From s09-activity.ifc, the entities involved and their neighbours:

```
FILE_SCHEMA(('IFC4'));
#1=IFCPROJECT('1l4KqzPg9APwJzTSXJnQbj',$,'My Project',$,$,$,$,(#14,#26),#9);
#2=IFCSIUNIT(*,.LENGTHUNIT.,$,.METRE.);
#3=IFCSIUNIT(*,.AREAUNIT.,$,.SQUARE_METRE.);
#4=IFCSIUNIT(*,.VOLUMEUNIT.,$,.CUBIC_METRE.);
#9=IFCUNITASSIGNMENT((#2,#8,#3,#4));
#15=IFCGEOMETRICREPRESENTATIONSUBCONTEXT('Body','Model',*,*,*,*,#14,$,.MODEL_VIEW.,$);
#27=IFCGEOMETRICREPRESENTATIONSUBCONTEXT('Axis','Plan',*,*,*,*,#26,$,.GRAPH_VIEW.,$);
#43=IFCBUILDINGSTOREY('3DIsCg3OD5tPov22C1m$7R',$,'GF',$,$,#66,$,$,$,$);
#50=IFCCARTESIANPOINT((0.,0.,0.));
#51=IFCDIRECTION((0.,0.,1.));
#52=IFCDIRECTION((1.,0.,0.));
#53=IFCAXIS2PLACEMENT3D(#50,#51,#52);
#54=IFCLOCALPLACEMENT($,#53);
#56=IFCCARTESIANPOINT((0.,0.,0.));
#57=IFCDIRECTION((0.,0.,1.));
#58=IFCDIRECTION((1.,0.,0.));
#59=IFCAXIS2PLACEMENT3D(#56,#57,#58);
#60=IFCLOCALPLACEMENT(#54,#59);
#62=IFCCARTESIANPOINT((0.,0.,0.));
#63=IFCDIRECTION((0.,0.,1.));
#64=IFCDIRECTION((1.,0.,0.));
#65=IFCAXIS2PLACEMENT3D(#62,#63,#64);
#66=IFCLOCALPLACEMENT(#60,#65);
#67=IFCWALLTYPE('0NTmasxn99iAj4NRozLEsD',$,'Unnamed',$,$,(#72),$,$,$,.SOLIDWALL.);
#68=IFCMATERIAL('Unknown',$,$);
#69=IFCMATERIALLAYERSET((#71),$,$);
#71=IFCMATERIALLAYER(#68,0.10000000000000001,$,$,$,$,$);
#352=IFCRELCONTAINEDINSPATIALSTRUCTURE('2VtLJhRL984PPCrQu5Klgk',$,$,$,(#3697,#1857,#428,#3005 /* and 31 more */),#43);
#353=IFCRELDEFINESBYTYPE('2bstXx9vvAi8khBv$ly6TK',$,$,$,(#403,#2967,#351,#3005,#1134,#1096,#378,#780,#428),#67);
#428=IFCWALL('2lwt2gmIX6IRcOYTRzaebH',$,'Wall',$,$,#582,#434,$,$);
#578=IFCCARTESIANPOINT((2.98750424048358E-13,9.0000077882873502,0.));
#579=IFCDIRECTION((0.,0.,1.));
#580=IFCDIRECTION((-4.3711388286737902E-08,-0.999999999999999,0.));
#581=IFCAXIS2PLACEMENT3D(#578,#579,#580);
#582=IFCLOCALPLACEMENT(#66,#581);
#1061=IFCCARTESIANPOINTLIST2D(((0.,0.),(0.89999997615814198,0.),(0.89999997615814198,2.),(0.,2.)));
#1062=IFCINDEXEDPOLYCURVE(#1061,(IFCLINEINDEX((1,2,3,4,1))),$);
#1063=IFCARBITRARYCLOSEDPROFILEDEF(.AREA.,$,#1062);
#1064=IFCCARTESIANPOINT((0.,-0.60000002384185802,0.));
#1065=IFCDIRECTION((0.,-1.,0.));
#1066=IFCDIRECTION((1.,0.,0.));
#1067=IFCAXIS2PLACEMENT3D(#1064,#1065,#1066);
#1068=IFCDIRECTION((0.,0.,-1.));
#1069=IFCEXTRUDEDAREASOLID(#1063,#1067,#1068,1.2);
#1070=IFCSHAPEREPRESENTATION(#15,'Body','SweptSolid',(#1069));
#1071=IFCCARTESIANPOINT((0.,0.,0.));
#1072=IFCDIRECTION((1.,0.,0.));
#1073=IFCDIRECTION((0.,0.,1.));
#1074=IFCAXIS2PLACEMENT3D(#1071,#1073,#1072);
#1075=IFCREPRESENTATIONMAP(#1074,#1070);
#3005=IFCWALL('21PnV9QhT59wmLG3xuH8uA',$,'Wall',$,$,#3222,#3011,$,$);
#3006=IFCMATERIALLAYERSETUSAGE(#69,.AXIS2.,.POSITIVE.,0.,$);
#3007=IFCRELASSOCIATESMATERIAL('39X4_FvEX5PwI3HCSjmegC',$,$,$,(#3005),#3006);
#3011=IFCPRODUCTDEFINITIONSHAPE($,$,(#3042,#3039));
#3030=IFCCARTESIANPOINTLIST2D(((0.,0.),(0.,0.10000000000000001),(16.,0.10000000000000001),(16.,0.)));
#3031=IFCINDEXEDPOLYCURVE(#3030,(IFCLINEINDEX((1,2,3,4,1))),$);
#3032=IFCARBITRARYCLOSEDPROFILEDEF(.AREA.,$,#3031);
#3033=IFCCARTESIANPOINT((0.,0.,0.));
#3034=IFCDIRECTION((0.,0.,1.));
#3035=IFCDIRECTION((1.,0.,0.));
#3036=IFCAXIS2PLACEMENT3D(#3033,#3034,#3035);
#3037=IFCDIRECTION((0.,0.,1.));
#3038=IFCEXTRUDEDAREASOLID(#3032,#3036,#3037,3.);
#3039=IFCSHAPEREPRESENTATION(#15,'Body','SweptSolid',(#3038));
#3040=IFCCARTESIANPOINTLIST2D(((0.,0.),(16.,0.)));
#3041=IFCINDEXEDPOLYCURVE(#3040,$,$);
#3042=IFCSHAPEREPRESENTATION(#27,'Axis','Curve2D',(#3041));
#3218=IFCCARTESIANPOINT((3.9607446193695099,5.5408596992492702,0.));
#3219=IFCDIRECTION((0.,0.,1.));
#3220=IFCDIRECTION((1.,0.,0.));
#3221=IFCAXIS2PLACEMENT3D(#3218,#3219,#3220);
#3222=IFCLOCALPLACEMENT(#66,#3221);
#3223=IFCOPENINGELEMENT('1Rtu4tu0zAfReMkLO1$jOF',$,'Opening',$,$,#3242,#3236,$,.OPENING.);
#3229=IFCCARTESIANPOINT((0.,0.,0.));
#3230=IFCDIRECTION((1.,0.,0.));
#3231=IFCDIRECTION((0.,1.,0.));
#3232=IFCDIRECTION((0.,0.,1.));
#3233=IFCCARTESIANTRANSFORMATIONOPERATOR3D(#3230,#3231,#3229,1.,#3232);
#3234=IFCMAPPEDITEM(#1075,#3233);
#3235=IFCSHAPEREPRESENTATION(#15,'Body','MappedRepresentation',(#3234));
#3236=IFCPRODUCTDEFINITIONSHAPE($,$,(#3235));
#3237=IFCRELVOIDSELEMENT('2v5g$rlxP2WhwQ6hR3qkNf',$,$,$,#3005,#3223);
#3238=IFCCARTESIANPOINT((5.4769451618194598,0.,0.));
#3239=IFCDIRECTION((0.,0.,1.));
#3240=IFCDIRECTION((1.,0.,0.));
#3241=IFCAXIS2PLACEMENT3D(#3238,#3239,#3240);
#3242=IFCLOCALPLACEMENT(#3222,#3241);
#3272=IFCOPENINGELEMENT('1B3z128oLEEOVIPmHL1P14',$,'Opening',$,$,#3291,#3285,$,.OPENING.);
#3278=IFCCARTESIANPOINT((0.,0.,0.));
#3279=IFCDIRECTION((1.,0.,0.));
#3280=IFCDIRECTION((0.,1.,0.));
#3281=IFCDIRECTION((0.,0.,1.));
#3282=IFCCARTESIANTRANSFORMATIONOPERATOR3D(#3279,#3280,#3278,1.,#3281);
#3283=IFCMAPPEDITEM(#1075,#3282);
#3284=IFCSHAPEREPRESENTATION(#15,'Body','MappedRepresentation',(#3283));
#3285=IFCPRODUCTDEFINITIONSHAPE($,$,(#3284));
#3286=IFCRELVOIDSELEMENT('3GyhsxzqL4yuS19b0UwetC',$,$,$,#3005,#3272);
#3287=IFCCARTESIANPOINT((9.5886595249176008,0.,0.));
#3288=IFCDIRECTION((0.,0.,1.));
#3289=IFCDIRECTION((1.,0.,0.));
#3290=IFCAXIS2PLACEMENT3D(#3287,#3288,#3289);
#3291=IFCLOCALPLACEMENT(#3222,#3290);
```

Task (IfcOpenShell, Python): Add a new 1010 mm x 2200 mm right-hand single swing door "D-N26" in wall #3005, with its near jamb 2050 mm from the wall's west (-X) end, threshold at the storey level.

```python
import numpy as np
import ifcopenshell
import ifcopenshell.api.feature
import ifcopenshell.api.geometry
import ifcopenshell.api.root
import ifcopenshell.api.spatial
import ifcopenshell.geom
import ifcopenshell.util.element
import ifcopenshell.util.placement
import ifcopenshell.util.representation
import ifcopenshell.util.shape
import ifcopenshell.util.unit

model = ifcopenshell.open("s09-activity.ifc")
unit_scale = ifcopenshell.util.unit.calculate_unit_scale(model)
settings = ifcopenshell.geom.settings()


def volume(element):
    """Net volume in cubic metres, openings subtracted."""
    shape = ifcopenshell.geom.create_shape(settings, element)
    return ifcopenshell.util.shape.get_volume(shape.geometry)


wall = model.by_guid("21PnV9QhT59wmLG3xuH8uA")
storey = ifcopenshell.util.element.get_container(wall, ifc_class="IfcBuildingStorey")
context = ifcopenshell.util.representation.get_context(model, "Model", "Body", "MODEL_VIEW")
before = volume(wall)

width, height, from_end, sill = 1.01, 2.2, 2.05, 0.0  # metres

# The wall runs along its own X axis, and the end named is its -X end.
wall_shape = ifcopenshell.geom.create_shape(settings, wall)
x, y, z = ifcopenshell.util.shape.get_vertices(wall_shape.geometry).T
start = x.min() + from_end
face, thickness = float(y.min()), float(y.max() - y.min())
wall_matrix = ifcopenshell.util.placement.get_local_placement(wall.ObjectPlacement)
level = ifcopenshell.util.placement.get_local_placement(storey.ObjectPlacement)[2, 3]


def in_wall(x, y):
    """Placement at x, y metres in the wall's axes, at sill height."""
    matrix = wall_matrix.copy()
    matrix[:, 3] = wall_matrix @ np.array([x / unit_scale, y / unit_scale, 0.0, 1.0])
    matrix[2, 3] = level + sill / unit_scale
    return matrix


# Opening: a box that overshoots both wall faces by 50 mm.
opening = ifcopenshell.api.root.create_entity(model, ifc_class="IfcOpeningElement", predefined_type="OPENING")
box = ifcopenshell.api.geometry.add_wall_representation(
    model, context=context, length=width, height=height, thickness=thickness + 0.1
)
ifcopenshell.api.geometry.assign_representation(model, product=opening, representation=box)
ifcopenshell.api.geometry.edit_object_placement(model, product=opening, matrix=in_wall(start, face - 0.05), is_si=False)
ifcopenshell.api.feature.add_feature(model, feature=opening, element=wall)

door = ifcopenshell.api.root.create_entity(model, ifc_class="IfcDoor", name="D-N26", predefined_type="DOOR")
door.OverallWidth, door.OverallHeight = width / unit_scale, height / unit_scale
door.OperationType = "SINGLE_SWING_RIGHT"
body = ifcopenshell.api.geometry.add_door_representation(
    model,
    context=context,
    overall_width=door.OverallWidth,
    overall_height=door.OverallHeight,
    operation_type="SINGLE_SWING_RIGHT",
    lining_properties={"LiningDepth": thickness / unit_scale, "ThresholdDepth": thickness / unit_scale},
)
ifcopenshell.api.geometry.assign_representation(model, product=door, representation=body)
ifcopenshell.api.spatial.assign_container(model, products=[door], relating_structure=storey)
ifcopenshell.api.feature.add_filling(model, opening=opening, element=door)

# The lining spans the wall, so the door starts at the wall face.
ifcopenshell.api.geometry.edit_object_placement(model, product=door, matrix=in_wall(start, face), is_si=False)

after = volume(wall)

print(f"wall volume {before:.3f} -> {after:.3f} m3")

model.write("s09-activity_rev.ifc")
```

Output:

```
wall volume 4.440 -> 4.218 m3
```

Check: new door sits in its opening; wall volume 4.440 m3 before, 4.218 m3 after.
